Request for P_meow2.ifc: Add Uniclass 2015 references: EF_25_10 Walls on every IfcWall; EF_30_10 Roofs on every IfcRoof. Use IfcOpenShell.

First a look at what the model holds.

```python
import ifcopenshell

model = ifcopenshell.open("P_meow2.ifc")
print(model.schema)
print("classifications:", [c.Name for c in model.by_type("IfcClassification")])
for ifc_class in ("IfcDoor", "IfcRoof", "IfcStair", "IfcWall", "IfcWindow"):
    print(ifc_class, len(model.by_type(ifc_class)))
```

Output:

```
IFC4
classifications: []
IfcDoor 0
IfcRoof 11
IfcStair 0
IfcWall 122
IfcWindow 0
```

```python
import ifcopenshell
import ifcopenshell.api.classification

model = ifcopenshell.open("P_meow2.ifc")

system = ifcopenshell.api.classification.add_classification(model, classification="Uniclass 2015")

codes = {
    "IfcWall": ("EF_25_10", "Walls"),
    "IfcRoof": ("EF_30_10", "Roofs"),
}
for ifc_class, (code, name) in codes.items():
    products = model.by_type(ifc_class)
    ifcopenshell.api.classification.add_reference(
        model, products=products, classification=system, identification=code, name=name
    )
    print(code, len(products))

model.write("P_meow2_rev.ifc")
```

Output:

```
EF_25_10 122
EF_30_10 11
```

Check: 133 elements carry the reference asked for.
